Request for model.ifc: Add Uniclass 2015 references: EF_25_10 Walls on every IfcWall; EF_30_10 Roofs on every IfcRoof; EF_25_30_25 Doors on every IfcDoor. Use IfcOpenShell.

First a look at what the model holds.

```python
import ifcopenshell

model = ifcopenshell.open("model.ifc")
print(model.schema)
print("classifications:", [c.Name for c in model.by_type("IfcClassification")])
for ifc_class in ("IfcDoor", "IfcRoof", "IfcStair", "IfcWall", "IfcWindow"):
    print(ifc_class, len(model.by_type(ifc_class)))
```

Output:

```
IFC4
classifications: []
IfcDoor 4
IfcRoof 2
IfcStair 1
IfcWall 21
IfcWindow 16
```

```python
import ifcopenshell
import ifcopenshell.api.classification

model = ifcopenshell.open("model.ifc")

system = ifcopenshell.api.classification.add_classification(model, classification="Uniclass 2015")

codes = {
    "IfcWall": ("EF_25_10", "Walls"),
    "IfcRoof": ("EF_30_10", "Roofs"),
    "IfcDoor": ("EF_25_30_25", "Doors"),
}
for ifc_class, (code, name) in codes.items():
    products = model.by_type(ifc_class)
    ifcopenshell.api.classification.add_reference(
        model, products=products, classification=system, identification=code, name=name
    )
    print(code, len(products))

model.write("model_edited.ifc")
```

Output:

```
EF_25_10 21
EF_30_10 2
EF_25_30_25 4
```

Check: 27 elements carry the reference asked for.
